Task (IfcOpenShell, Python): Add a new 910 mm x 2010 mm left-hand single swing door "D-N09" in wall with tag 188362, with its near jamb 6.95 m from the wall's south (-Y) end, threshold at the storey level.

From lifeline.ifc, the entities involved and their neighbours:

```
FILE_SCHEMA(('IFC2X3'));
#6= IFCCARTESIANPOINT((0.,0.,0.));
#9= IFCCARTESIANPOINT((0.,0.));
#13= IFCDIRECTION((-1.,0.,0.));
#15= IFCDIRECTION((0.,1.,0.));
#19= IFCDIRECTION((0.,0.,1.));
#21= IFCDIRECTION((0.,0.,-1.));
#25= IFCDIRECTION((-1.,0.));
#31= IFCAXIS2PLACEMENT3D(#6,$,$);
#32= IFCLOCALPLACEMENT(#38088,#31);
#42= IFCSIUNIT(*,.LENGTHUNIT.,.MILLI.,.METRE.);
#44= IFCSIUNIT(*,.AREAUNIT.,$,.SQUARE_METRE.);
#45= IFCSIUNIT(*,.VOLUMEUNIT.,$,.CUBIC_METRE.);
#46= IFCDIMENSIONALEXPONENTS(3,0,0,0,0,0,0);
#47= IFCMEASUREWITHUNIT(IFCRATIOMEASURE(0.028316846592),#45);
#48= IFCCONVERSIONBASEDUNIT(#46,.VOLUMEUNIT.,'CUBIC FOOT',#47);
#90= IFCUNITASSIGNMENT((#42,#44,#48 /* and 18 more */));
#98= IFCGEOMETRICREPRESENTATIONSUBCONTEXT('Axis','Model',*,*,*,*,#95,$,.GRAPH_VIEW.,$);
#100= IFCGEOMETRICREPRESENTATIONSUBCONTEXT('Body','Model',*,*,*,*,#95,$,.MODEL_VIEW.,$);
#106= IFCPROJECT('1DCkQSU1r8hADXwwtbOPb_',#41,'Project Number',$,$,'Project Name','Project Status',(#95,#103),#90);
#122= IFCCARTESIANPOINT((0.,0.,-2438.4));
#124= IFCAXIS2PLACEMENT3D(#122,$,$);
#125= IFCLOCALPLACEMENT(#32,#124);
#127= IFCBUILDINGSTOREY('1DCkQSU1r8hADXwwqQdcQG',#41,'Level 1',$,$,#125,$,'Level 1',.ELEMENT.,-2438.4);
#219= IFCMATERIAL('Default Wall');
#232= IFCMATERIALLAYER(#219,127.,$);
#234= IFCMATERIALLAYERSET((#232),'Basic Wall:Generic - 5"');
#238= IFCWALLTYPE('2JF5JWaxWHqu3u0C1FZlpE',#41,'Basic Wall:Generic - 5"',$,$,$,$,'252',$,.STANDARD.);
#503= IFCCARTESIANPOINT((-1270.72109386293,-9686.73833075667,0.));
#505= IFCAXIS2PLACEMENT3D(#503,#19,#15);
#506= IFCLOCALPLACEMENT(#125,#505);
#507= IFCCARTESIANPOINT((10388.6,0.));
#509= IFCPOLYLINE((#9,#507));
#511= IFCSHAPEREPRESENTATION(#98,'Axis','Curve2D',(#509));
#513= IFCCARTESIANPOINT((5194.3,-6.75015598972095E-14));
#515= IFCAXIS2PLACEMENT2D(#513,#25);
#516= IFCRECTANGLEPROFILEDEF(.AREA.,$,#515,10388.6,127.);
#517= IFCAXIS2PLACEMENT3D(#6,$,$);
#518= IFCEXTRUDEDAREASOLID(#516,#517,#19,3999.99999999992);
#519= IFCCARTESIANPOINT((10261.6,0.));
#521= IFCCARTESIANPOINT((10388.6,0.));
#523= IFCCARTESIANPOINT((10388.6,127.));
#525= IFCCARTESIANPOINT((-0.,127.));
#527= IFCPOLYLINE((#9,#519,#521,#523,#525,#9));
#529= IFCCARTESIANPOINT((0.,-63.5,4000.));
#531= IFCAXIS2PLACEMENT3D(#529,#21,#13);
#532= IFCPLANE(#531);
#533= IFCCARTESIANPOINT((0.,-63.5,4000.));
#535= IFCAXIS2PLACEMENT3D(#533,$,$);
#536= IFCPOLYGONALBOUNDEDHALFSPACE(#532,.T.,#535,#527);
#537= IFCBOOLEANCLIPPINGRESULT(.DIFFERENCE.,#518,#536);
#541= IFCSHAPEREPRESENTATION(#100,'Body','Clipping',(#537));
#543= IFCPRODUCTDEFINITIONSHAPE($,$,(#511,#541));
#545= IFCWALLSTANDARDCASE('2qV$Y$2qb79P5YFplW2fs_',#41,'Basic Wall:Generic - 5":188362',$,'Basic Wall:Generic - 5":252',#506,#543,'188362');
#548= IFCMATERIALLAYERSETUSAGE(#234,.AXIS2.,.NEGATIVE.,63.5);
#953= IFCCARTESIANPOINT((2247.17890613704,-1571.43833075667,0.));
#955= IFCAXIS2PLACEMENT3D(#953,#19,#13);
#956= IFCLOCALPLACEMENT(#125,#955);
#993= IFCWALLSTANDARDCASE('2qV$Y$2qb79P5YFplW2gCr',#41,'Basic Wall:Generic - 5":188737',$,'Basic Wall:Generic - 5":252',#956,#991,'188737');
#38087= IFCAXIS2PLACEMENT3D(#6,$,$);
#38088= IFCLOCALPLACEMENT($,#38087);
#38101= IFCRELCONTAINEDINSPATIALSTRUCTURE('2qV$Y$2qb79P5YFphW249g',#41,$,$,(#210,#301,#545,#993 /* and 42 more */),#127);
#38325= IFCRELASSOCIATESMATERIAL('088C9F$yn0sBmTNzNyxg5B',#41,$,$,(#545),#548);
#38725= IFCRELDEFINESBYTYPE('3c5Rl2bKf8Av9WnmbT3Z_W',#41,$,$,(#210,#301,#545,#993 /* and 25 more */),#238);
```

```python
import numpy as np
import ifcopenshell
import ifcopenshell.api.feature
import ifcopenshell.api.geometry
import ifcopenshell.api.root
import ifcopenshell.api.spatial
import ifcopenshell.api.type
import ifcopenshell.geom
import ifcopenshell.util.element
import ifcopenshell.util.placement
import ifcopenshell.util.representation
import ifcopenshell.util.shape
import ifcopenshell.util.unit

model = ifcopenshell.open("lifeline.ifc")
unit_scale = ifcopenshell.util.unit.calculate_unit_scale(model)
settings = ifcopenshell.geom.settings()


def volume(element):
    """Net volume in cubic metres, openings subtracted."""
    shape = ifcopenshell.geom.create_shape(settings, element)
    return ifcopenshell.util.shape.get_volume(shape.geometry)


wall = model.by_guid("2qV$Y$2qb79P5YFplW2fs_")
storey = ifcopenshell.util.element.get_container(wall, ifc_class="IfcBuildingStorey")
context = ifcopenshell.util.representation.get_context(model, "Model", "Body", "MODEL_VIEW")
before = volume(wall)

width, height, from_end, sill = 0.91, 2.01, 6.95, 0.0  # metres

# The wall runs along its own X axis, and the end named is its -X end.
wall_shape = ifcopenshell.geom.create_shape(settings, wall)
x, y, z = ifcopenshell.util.shape.get_vertices(wall_shape.geometry).T
start = x.min() + from_end
face, thickness = float(y.min()), float(y.max() - y.min())
wall_matrix = ifcopenshell.util.placement.get_local_placement(wall.ObjectPlacement)
level = ifcopenshell.util.placement.get_local_placement(storey.ObjectPlacement)[2, 3]


def in_wall(x, y):
    """Placement at x, y metres in the wall's axes, at sill height."""
    matrix = wall_matrix.copy()
    matrix[:, 3] = wall_matrix @ np.array([x / unit_scale, y / unit_scale, 0.0, 1.0])
    matrix[2, 3] = level + sill / unit_scale
    return matrix


# Opening: a box that overshoots both wall faces by 50 mm.
opening = ifcopenshell.api.root.create_entity(model, ifc_class="IfcOpeningElement")
box = ifcopenshell.api.geometry.add_wall_representation(
    model, context=context, length=width, height=height, thickness=thickness + 0.1
)
ifcopenshell.api.geometry.assign_representation(model, product=opening, representation=box)
ifcopenshell.api.geometry.edit_object_placement(model, product=opening, matrix=in_wall(start, face - 0.05), is_si=False)
ifcopenshell.api.feature.add_feature(model, feature=opening, element=wall)

door = ifcopenshell.api.root.create_entity(model, ifc_class="IfcDoor", name="D-N09")
door.OverallWidth, door.OverallHeight = width / unit_scale, height / unit_scale
body = ifcopenshell.api.geometry.add_door_representation(
    model,
    context=context,
    overall_width=door.OverallWidth,
    overall_height=door.OverallHeight,
    operation_type="SINGLE_SWING_LEFT",
    lining_properties={"LiningDepth": thickness / unit_scale, "ThresholdDepth": thickness / unit_scale},
)
ifcopenshell.api.geometry.assign_representation(model, product=door, representation=body)
ifcopenshell.api.spatial.assign_container(model, products=[door], relating_structure=storey)
fills = ifcopenshell.api.feature.add_filling(model, opening=opening, element=door)
fills.OwnerHistory = door.OwnerHistory  # required in IFC2X3

# IFC2X3 keeps the operation on the door style.
style = ifcopenshell.api.root.create_entity(model, ifc_class="IfcDoorStyle", name="D-N09")
style.OperationType, style.ConstructionType = "SINGLE_SWING_LEFT", "NOTDEFINED"
style.ParameterTakesPrecedence = style.Sizeable = False
ifcopenshell.api.type.assign_type(model, related_objects=[door], relating_type=style)

# The lining spans the wall, so the door starts at the wall face.
ifcopenshell.api.geometry.edit_object_placement(model, product=door, matrix=in_wall(start, face), is_si=False)

after = volume(wall)

print(f"wall volume {before:.3f} -> {after:.3f} m3")

model.write("lifeline-out.ifc")
```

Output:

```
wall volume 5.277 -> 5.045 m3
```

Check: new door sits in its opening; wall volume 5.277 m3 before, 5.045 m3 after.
